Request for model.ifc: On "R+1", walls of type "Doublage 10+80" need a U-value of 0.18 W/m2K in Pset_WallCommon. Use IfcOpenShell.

First a look at what the model holds.

```python
import ifcopenshell
import ifcopenshell.util.element

model = ifcopenshell.open("model.ifc")
print(model.schema)
storey = next(s for s in model.by_type("IfcBuildingStorey") if s.Name == "R+1")
walls = [e for e in ifcopenshell.util.element.get_decomposition(storey) if e.is_a("IfcWall")]
seen = {}
for e in walls:
    element_type = ifcopenshell.util.element.get_type(e)
    key = (element_type.Name if element_type != e and element_type else None, ifcopenshell.util.element.get_pset(e, "Pset_WallCommon", "ThermalTransmittance"))
    seen[key] = seen.get(key, 0) + 1
for (name, value), count in sorted(seen.items(), key=str):
    print(count, "x", name, "|", value)
```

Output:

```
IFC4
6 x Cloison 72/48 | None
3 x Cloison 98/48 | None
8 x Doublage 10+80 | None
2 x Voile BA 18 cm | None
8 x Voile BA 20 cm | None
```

```python
import ifcopenshell
import ifcopenshell.api.pset
import ifcopenshell.util.element

model = ifcopenshell.open("model.ifc")

storey = next(s for s in model.by_type("IfcBuildingStorey") if s.Name == "R+1")
walls = [e for e in ifcopenshell.util.element.get_decomposition(storey) if e.is_a("IfcWall")]

count = 0
for e in walls:
    element_type = ifcopenshell.util.element.get_type(e)
    if element_type in (None, e) or element_type.Name != "Doublage 10+80":
        continue
    # add_pset returns the element's existing set when there is one.
    pset = ifcopenshell.api.pset.add_pset(model, product=e, name="Pset_WallCommon")
    ifcopenshell.api.pset.edit_pset(model, pset=pset, properties={"ThermalTransmittance": 0.18})
    count += 1

print(count, "walls updated")

model.write("model-out.ifc")
```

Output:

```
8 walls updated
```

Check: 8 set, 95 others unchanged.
